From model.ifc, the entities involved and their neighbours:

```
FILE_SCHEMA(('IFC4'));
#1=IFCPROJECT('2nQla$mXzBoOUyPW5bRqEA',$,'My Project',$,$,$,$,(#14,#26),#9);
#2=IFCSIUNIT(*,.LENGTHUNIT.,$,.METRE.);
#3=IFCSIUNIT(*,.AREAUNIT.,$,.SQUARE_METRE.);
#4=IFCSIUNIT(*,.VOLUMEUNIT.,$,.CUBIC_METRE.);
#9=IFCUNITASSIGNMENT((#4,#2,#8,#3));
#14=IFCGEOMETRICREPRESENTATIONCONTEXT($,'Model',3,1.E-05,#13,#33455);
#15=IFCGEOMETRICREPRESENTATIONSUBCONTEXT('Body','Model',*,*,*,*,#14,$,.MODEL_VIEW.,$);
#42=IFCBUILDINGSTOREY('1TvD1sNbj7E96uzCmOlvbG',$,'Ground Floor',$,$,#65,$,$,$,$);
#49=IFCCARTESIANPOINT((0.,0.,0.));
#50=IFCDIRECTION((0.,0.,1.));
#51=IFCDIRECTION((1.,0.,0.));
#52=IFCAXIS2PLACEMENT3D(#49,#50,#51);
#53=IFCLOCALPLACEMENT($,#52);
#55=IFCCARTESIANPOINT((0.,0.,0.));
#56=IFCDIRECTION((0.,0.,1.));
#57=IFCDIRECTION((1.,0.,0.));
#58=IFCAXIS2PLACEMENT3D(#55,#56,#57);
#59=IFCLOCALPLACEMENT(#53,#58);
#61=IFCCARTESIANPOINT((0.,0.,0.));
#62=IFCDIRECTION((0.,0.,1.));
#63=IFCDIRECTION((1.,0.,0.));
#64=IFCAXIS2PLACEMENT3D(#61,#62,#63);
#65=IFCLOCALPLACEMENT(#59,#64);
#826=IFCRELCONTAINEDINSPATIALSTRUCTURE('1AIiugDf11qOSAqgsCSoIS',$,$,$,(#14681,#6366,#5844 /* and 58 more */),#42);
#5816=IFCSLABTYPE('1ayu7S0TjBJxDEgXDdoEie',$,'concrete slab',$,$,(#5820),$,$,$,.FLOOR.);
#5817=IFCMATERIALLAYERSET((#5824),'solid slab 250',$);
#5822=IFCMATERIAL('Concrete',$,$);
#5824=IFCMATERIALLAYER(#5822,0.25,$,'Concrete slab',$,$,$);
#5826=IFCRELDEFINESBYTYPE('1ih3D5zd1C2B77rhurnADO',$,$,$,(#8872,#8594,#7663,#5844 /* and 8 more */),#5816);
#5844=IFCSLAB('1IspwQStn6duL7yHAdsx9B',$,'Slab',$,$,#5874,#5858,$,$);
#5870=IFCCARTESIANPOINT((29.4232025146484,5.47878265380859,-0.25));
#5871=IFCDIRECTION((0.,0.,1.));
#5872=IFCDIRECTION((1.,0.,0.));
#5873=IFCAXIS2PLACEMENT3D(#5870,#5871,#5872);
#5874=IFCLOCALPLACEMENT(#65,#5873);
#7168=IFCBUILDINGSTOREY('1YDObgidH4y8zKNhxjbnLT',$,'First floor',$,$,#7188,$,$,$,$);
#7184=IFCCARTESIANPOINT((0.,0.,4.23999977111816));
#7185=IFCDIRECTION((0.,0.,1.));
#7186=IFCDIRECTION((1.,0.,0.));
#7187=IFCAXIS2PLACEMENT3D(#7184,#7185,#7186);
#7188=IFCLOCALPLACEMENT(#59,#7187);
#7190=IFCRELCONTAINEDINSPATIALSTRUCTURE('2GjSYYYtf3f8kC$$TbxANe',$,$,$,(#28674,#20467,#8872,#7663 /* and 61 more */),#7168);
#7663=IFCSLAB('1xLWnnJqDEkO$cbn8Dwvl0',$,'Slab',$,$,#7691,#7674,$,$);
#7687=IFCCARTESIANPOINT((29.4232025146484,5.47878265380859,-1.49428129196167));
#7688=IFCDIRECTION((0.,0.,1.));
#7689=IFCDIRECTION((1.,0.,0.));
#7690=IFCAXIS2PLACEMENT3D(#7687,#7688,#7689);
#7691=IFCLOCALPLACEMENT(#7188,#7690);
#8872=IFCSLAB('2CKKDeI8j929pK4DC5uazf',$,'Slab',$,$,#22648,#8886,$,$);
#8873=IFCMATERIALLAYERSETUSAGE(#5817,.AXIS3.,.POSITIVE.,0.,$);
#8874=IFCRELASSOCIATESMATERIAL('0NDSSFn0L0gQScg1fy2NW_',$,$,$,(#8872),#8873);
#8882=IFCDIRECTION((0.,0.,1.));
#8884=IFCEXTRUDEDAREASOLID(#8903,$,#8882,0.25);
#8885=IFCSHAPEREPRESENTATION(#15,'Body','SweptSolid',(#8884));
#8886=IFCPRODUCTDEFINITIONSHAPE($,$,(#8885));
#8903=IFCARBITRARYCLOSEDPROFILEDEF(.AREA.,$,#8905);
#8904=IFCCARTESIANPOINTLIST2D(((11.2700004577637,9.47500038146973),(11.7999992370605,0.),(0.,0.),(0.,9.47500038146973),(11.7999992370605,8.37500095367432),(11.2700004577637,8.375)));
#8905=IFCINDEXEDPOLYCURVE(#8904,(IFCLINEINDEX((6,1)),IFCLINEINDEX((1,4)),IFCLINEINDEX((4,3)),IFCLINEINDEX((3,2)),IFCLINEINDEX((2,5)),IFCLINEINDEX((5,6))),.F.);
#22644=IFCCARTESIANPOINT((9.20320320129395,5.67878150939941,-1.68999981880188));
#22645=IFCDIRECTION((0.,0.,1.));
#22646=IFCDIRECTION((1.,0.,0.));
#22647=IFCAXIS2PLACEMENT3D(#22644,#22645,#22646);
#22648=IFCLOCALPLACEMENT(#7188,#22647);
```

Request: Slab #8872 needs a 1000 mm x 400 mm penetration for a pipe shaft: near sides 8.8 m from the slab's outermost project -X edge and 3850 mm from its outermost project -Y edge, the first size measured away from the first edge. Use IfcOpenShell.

```python
import numpy as np
import ifcopenshell
import ifcopenshell.api.feature
import ifcopenshell.api.geometry
import ifcopenshell.api.root
import ifcopenshell.geom
import ifcopenshell.util.placement
import ifcopenshell.util.representation
import ifcopenshell.util.shape
import ifcopenshell.util.unit

model = ifcopenshell.open("model.ifc")
unit_scale = ifcopenshell.util.unit.calculate_unit_scale(model)
settings = ifcopenshell.geom.settings()


def volume(element):
    """Net volume in cubic metres, openings subtracted."""
    shape = ifcopenshell.geom.create_shape(settings, element)
    return ifcopenshell.util.shape.get_volume(shape.geometry)


slab = model.by_id(8872)
before = volume(slab)

# Extent in the slab's own axes, in metres. The edges named are its -X and -Y sides.
slab_shape = ifcopenshell.geom.create_shape(settings, slab)
vertices = ifcopenshell.util.shape.get_vertices(slab_shape.geometry)
x_min, y_min, bottom = vertices.min(axis=0)
top = vertices[:, 2].max()

opening = ifcopenshell.api.root.create_entity(model, ifc_class="IfcOpeningElement", name="Pipe shaft opening", predefined_type="OPENING")
context = ifcopenshell.util.representation.get_context(model, "Model", "Body", "MODEL_VIEW")
width, depth = 1, 0.4
outline = [(0.0, 0.0), (width, 0.0), (width, depth), (0.0, depth), (0.0, 0.0)]
# Overshoot both faces by 50 mm so the cut is clean.
shape = ifcopenshell.api.geometry.add_slab_representation(
    model, context=context, depth=top - bottom + 0.1, polyline=outline
)
ifcopenshell.api.geometry.assign_representation(model, product=opening, representation=shape)

matrix = ifcopenshell.util.placement.get_local_placement(slab.ObjectPlacement)
matrix[:, 3] = matrix @ np.append(np.array([x_min + 8.8, y_min + 3.85, bottom - 0.05]) / unit_scale, 1.0)
ifcopenshell.api.geometry.edit_object_placement(model, product=opening, matrix=matrix, is_si=False)
ifcopenshell.api.feature.add_feature(model, feature=opening, element=slab)

after = volume(slab)

print(f"slab volume {before:.3f} -> {after:.3f} m3")

model.write("model_edited.ifc")
```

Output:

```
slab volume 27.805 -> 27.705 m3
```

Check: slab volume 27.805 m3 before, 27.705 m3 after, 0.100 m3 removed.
